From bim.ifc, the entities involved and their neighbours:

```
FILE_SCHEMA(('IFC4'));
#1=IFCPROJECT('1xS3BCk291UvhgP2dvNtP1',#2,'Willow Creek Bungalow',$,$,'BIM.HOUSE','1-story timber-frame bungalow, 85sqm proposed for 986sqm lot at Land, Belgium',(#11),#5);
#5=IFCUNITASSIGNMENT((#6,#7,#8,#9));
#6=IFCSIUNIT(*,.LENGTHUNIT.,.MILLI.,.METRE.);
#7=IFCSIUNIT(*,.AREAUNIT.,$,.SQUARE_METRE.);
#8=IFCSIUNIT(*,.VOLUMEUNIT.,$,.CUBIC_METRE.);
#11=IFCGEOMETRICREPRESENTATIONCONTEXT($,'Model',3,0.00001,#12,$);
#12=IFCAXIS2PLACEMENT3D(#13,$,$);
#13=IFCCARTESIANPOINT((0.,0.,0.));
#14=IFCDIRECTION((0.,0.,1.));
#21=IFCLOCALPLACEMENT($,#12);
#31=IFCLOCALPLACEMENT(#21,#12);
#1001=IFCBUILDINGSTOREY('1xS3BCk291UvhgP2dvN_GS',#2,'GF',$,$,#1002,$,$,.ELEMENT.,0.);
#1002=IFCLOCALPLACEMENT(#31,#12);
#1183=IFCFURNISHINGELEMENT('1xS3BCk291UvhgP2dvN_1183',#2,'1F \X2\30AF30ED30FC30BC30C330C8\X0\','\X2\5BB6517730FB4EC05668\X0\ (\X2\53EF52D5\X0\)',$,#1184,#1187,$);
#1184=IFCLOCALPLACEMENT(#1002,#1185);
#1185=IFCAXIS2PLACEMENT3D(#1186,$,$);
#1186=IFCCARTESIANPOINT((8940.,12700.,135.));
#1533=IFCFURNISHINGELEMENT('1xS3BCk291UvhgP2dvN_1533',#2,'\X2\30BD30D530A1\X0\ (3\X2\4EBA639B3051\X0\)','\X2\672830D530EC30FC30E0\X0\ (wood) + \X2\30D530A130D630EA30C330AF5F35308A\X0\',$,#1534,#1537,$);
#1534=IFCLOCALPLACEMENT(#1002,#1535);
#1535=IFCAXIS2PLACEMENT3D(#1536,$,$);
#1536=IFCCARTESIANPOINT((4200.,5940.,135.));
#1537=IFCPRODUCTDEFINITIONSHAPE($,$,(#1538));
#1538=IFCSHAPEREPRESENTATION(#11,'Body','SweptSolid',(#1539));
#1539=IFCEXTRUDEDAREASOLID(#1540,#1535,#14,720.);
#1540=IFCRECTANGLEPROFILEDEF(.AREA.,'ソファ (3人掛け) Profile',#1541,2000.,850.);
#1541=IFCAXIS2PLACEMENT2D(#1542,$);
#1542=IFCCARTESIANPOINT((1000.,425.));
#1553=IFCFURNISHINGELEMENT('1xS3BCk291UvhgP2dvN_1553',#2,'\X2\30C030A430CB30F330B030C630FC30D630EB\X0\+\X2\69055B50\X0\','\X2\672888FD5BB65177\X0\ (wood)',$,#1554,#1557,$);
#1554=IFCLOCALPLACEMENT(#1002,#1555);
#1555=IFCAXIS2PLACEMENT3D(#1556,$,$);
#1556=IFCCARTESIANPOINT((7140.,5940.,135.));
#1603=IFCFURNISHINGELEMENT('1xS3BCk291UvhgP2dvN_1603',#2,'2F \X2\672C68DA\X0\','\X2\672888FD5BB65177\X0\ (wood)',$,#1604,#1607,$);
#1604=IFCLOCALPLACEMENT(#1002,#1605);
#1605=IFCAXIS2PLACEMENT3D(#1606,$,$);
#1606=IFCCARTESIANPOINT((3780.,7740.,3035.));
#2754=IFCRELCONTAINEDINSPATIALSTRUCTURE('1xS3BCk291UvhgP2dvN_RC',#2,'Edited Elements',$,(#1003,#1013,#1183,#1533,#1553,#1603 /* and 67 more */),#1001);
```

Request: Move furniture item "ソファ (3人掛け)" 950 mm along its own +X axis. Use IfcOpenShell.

```python
import ifcopenshell
import ifcopenshell.api.geometry
import ifcopenshell.util.placement
import ifcopenshell.util.unit

model = ifcopenshell.open("bim.ifc")
unit_scale = ifcopenshell.util.unit.calculate_unit_scale(model)

item = model.by_guid("1xS3BCk291UvhgP2dvN_1533")
matrix = ifcopenshell.util.placement.get_local_placement(item.ObjectPlacement)
matrix[:3, 3] += matrix[:3, 0] * 0.95 / unit_scale
ifcopenshell.api.geometry.edit_object_placement(model, product=item, matrix=matrix, is_si=False)

print(ifcopenshell.util.placement.get_local_placement(item.ObjectPlacement).round(3) + 0.0)

model.write("bim_edited.ifc")
```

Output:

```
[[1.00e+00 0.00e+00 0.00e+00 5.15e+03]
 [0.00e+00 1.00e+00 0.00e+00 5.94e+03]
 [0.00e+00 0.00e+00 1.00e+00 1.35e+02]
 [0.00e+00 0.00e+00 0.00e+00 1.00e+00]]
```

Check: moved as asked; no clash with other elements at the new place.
